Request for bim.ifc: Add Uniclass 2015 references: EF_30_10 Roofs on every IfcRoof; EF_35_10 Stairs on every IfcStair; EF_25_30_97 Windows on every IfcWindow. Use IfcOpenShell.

First a look at what the model holds.

```python
import ifcopenshell

model = ifcopenshell.open("bim.ifc")
print(model.schema)
print("classifications:", [c.Name for c in model.by_type("IfcClassification")])
for ifc_class in ("IfcDoor", "IfcRoof", "IfcStair", "IfcWall", "IfcWindow"):
    print(ifc_class, len(model.by_type(ifc_class)))
```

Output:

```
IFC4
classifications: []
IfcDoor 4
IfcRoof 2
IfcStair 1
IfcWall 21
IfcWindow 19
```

```python
import ifcopenshell
import ifcopenshell.api.classification

model = ifcopenshell.open("bim.ifc")

system = ifcopenshell.api.classification.add_classification(model, classification="Uniclass 2015")

codes = {
    "IfcRoof": ("EF_30_10", "Roofs"),
    "IfcStair": ("EF_35_10", "Stairs"),
    "IfcWindow": ("EF_25_30_97", "Windows"),
}
for ifc_class, (code, name) in codes.items():
    products = model.by_type(ifc_class)
    ifcopenshell.api.classification.add_reference(
        model, products=products, classification=system, identification=code, name=name
    )
    print(code, len(products))

model.write("bim_v2.ifc")
```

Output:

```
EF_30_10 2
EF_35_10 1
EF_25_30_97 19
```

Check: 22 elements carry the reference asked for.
